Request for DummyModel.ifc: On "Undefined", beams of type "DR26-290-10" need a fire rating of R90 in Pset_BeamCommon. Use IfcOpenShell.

First a look at what the model holds.

```python
import ifcopenshell
import ifcopenshell.util.element

model = ifcopenshell.open("DummyModel.ifc")
print(model.schema)
storey = next(s for s in model.by_type("IfcBuildingStorey") if s.Name == "Undefined")
beams = [e for e in ifcopenshell.util.element.get_decomposition(storey) if e.is_a("IfcBeam")]
seen = {}
for e in beams:
    element_type = ifcopenshell.util.element.get_type(e)
    key = (element_type.Name if element_type != e and element_type else None, ifcopenshell.util.element.get_pset(e, "Pset_BeamCommon", "FireRating"))
    seen[key] = seen.get(key, 0) + 1
for (name, value), count in sorted(seen.items(), key=str):
    print(count, "x", name, "|", value)
```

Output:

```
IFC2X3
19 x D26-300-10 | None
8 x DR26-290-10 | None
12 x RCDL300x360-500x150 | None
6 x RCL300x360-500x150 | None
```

```python
import ifcopenshell
import ifcopenshell.api.pset
import ifcopenshell.util.element

model = ifcopenshell.open("DummyModel.ifc")

storey = next(s for s in model.by_type("IfcBuildingStorey") if s.Name == "Undefined")
beams = [e for e in ifcopenshell.util.element.get_decomposition(storey) if e.is_a("IfcBeam")]

count = 0
for e in beams:
    element_type = ifcopenshell.util.element.get_type(e)
    if element_type in (None, e) or element_type.Name != "DR26-290-10":
        continue
    found = ifcopenshell.util.element.get_pset(e, "Pset_BeamCommon", should_inherit=False)
    if found:
        pset = model.by_id(found["id"])
        if len(ifcopenshell.util.element.get_elements_by_pset(pset)) > 1:
            pset = ifcopenshell.api.pset.unshare_pset(model, products=[e], pset=pset)[0]
    else:
        pset = ifcopenshell.api.pset.add_pset(model, product=e, name="Pset_BeamCommon")
    ifcopenshell.api.pset.edit_pset(model, pset=pset, properties={"FireRating": "R90"})
    count += 1

print(count, "beams updated")

model.write("DummyModel-out.ifc")
```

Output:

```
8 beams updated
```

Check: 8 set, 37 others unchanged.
